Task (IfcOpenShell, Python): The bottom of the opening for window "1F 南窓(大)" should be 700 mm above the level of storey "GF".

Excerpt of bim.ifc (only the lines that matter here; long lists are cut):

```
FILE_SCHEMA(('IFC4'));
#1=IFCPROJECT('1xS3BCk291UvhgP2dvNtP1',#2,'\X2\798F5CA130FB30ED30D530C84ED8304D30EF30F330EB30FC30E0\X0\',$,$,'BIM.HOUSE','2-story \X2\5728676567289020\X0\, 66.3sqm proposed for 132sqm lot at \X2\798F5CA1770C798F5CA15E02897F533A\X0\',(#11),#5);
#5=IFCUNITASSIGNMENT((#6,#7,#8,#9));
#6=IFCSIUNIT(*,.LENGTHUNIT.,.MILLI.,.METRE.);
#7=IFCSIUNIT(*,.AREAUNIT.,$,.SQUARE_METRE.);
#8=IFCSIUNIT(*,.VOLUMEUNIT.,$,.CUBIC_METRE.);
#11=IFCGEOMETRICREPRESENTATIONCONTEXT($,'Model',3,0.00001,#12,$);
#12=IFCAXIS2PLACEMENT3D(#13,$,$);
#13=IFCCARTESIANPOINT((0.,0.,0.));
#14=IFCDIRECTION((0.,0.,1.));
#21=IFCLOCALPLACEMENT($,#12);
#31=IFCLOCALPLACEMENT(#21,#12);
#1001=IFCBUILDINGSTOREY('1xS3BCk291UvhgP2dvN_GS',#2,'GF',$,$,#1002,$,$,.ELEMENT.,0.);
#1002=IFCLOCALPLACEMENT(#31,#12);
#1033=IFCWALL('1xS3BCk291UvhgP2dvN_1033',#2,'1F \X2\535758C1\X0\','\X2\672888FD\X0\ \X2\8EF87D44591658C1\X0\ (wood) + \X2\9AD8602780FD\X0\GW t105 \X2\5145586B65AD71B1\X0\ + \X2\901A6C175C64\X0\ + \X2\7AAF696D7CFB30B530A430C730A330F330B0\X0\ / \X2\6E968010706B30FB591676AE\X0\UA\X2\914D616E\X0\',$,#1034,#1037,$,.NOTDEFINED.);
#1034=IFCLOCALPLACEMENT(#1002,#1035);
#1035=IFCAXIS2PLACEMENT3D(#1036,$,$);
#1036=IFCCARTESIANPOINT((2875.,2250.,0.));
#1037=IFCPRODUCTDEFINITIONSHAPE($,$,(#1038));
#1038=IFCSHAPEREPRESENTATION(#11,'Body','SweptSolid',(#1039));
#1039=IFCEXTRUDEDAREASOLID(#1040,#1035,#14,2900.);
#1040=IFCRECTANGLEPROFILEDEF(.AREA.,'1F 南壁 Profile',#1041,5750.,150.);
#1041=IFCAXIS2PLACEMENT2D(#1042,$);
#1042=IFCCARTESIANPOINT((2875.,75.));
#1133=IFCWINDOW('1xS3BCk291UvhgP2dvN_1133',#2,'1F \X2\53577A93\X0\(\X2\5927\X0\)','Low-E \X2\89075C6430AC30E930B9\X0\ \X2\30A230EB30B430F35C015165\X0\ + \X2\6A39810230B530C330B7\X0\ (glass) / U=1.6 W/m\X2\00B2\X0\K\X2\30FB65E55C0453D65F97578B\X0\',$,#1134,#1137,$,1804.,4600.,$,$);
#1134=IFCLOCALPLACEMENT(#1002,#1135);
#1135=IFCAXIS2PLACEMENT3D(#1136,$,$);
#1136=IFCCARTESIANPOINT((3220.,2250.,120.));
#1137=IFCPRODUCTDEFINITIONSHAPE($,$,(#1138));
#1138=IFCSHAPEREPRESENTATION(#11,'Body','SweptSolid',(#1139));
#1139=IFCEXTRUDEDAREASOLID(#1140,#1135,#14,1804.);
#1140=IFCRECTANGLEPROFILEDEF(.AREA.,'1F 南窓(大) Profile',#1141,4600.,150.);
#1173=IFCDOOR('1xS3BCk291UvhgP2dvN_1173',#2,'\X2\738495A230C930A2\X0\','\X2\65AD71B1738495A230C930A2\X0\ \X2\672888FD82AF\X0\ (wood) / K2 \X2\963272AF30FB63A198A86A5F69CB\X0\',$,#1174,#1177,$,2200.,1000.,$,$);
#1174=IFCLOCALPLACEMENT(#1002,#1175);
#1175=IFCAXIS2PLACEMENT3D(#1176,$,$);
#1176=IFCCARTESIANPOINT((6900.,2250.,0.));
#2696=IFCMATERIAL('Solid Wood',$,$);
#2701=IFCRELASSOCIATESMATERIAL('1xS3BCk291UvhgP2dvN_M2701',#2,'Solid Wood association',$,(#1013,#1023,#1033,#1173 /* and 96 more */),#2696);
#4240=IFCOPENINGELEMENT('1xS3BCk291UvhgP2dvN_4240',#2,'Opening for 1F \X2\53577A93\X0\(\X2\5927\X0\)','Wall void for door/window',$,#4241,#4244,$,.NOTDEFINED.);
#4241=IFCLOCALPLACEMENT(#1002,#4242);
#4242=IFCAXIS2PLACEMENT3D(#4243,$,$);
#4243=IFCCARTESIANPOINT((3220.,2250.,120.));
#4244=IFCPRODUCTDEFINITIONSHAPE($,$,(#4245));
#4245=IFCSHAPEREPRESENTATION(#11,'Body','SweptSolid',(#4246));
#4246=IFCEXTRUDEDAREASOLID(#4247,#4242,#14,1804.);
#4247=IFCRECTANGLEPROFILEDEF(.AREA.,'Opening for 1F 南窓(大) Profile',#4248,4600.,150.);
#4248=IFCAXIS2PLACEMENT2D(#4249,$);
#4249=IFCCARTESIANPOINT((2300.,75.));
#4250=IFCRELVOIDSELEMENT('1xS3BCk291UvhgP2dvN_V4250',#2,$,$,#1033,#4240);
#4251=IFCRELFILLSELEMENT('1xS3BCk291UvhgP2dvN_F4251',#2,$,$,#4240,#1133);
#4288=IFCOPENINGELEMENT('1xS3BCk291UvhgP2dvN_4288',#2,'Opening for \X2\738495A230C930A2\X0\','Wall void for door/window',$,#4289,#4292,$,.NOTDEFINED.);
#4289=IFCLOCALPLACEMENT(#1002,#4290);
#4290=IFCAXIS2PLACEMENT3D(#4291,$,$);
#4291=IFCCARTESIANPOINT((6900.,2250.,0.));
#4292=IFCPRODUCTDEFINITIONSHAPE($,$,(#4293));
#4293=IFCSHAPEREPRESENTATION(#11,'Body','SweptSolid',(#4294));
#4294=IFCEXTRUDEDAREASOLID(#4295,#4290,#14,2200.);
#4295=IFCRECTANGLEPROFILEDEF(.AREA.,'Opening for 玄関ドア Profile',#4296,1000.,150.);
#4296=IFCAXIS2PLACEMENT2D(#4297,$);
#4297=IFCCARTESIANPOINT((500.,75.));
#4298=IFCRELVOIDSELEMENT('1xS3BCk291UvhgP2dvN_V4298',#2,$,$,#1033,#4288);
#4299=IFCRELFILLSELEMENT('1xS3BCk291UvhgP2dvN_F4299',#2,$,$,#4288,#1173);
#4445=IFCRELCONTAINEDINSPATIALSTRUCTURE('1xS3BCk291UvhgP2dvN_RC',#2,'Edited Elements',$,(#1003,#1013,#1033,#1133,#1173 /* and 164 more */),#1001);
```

```python
import numpy as np
import ifcopenshell
import ifcopenshell.api.geometry
import ifcopenshell.geom
import ifcopenshell.util.element
import ifcopenshell.util.placement
import ifcopenshell.util.shape
import ifcopenshell.util.unit

model = ifcopenshell.open("bim.ifc")
unit_scale = ifcopenshell.util.unit.calculate_unit_scale(model)

window = model.by_guid("1xS3BCk291UvhgP2dvN_1133")
opening = window.FillsVoids[0].RelatingOpeningElement
storey = ifcopenshell.util.element.get_container(window, ifc_class="IfcBuildingStorey")
level = ifcopenshell.util.placement.get_local_placement(storey.ObjectPlacement)[2, 3]

# The opening's origin need not be at the sill, so measure its lowest point.
shape = ifcopenshell.geom.create_shape(ifcopenshell.geom.settings(), opening)
bottom = ifcopenshell.util.shape.get_shape_bottom_elevation(shape, shape.geometry) / unit_scale
dz = level + 0.7 / unit_scale - bottom

shift = np.array([0.0, 0.0, dz])
# The window is not placed relative to its opening, so move both.
for product in (opening, window):
    matrix = ifcopenshell.util.placement.get_local_placement(product.ObjectPlacement)
    matrix[:3, 3] += shift
    ifcopenshell.api.geometry.edit_object_placement(model, product=product, matrix=matrix, is_si=False)

print(f"moved by {dz * unit_scale:+.3f} m")

model.write("bim_updated.ifc")
```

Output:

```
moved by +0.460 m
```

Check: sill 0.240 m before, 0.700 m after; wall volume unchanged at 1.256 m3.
